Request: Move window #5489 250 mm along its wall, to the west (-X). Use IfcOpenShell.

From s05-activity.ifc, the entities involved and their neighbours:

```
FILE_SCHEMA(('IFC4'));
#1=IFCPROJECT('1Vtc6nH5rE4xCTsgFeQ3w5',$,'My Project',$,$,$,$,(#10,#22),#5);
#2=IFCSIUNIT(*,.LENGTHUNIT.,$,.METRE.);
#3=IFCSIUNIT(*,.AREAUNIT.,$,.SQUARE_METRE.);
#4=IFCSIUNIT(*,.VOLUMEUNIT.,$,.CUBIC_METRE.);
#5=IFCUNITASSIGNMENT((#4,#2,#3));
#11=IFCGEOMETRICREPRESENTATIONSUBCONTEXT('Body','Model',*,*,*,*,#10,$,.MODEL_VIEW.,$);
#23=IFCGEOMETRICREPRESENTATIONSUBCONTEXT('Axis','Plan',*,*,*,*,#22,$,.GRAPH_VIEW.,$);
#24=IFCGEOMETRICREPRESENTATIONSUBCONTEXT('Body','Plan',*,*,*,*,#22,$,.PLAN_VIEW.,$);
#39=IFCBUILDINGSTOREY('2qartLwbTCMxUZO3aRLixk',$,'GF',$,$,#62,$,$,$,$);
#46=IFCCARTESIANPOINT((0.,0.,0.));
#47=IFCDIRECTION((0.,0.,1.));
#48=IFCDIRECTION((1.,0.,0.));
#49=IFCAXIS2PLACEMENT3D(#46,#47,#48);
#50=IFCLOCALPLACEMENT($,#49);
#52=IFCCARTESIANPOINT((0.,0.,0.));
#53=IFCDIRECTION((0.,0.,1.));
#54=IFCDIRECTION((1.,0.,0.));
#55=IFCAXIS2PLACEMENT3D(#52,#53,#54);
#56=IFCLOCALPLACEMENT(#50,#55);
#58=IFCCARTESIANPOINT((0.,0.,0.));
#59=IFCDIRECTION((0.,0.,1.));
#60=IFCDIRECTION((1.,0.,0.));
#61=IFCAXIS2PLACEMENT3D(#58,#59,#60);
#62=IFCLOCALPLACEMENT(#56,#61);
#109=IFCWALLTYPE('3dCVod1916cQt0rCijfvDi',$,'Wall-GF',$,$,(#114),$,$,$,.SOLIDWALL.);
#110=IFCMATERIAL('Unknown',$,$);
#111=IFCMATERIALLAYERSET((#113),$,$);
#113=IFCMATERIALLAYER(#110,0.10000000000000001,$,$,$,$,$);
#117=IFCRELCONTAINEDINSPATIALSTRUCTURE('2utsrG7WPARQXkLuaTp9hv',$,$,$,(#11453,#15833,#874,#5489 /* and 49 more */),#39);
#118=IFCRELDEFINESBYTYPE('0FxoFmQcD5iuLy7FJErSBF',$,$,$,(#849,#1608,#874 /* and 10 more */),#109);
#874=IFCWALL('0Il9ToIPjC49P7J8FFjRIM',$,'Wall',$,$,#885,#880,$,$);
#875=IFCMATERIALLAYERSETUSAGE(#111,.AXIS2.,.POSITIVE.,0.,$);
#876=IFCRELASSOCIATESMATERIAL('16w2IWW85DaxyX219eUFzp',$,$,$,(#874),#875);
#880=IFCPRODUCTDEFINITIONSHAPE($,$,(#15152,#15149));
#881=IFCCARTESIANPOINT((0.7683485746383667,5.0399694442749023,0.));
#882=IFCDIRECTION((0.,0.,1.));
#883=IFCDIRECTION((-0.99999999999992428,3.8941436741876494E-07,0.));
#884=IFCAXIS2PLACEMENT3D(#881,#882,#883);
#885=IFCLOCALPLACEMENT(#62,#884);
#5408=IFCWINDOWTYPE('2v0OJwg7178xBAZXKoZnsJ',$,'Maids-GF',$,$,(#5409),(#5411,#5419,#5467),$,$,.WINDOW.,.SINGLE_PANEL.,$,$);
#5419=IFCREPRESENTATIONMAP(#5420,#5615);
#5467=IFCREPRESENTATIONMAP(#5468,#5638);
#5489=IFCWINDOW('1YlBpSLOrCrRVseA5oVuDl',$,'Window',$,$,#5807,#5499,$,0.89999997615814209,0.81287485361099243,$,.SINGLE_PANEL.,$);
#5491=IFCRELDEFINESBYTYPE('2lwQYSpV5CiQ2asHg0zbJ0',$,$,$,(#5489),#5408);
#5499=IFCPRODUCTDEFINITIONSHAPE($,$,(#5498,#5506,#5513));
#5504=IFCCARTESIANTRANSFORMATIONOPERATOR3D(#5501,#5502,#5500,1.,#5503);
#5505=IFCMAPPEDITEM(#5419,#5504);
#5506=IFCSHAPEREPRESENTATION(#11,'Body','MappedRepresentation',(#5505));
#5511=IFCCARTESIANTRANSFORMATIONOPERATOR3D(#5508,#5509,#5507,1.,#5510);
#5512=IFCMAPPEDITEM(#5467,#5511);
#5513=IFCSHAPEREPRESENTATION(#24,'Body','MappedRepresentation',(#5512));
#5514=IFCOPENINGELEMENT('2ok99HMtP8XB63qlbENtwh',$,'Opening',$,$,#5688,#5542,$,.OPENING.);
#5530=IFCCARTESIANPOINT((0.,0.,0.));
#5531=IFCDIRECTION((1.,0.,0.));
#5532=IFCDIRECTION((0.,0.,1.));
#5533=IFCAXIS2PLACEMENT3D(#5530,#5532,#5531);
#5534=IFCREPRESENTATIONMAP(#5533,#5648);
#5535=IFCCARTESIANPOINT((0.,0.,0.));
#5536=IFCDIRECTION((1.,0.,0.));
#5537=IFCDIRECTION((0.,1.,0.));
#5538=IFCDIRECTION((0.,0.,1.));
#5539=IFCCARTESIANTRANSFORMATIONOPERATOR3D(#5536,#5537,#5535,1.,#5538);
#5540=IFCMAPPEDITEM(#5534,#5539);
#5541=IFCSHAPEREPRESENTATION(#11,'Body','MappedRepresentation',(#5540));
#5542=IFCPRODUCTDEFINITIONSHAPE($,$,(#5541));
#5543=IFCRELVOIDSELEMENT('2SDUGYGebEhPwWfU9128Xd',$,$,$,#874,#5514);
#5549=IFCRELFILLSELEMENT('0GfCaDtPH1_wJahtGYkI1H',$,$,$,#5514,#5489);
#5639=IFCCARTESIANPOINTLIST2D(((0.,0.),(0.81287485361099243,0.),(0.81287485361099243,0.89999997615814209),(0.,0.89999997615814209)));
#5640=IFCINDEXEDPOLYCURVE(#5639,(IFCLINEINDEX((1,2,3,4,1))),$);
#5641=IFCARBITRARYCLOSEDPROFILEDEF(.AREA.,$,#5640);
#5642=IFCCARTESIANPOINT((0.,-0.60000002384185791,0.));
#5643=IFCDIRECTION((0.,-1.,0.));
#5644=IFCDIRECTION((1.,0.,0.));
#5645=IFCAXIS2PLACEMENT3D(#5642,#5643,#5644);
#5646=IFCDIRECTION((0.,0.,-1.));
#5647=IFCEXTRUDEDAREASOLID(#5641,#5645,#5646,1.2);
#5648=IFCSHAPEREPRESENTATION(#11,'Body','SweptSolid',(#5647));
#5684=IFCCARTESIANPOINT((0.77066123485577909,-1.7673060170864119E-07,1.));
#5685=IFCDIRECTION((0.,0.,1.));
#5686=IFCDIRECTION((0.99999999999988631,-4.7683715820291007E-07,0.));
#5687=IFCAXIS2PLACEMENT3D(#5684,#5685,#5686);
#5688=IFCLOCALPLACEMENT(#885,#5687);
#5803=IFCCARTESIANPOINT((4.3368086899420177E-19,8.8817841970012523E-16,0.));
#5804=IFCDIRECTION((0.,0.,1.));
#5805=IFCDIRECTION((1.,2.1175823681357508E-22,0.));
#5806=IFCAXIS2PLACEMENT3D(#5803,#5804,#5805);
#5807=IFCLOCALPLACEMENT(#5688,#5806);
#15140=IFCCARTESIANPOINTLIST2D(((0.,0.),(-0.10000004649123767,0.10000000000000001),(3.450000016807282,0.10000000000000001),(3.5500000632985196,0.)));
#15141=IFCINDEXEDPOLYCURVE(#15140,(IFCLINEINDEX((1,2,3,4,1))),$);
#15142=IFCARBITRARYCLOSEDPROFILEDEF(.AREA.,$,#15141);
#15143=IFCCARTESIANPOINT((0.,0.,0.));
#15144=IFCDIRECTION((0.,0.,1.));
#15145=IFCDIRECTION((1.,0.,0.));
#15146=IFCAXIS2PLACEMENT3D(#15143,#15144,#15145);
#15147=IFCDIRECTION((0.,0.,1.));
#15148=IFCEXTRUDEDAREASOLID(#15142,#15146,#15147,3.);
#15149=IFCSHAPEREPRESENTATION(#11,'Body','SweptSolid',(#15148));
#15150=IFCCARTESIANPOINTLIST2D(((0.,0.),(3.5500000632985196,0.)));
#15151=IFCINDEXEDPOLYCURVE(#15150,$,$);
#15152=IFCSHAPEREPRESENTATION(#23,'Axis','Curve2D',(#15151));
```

```python
import ifcopenshell
import ifcopenshell.api.geometry
import ifcopenshell.util.placement

model = ifcopenshell.open("s05-activity.ifc")

window = model.by_guid("1YlBpSLOrCrRVseA5oVuDl")
opening = window.FillsVoids[0].RelatingOpeningElement
wall = opening.VoidsElements[0].RelatingBuildingElement

wall_matrix = ifcopenshell.util.placement.get_local_placement(wall.ObjectPlacement)
shift = wall_matrix[:3, 0] * 0.25
before = ifcopenshell.util.placement.get_local_placement(window.ObjectPlacement)[:3, 3].copy()

# The window is placed relative to its opening, so it follows when the opening moves.
matrix = ifcopenshell.util.placement.get_local_placement(opening.ObjectPlacement)
matrix[:3, 3] += shift
ifcopenshell.api.geometry.edit_object_placement(
    model, product=opening, matrix=matrix, is_si=False, should_transform_children=True
)

after = ifcopenshell.util.placement.get_local_placement(window.ObjectPlacement)[:3, 3]
print("window moved by", (after - before).round(3) + 0.0)

model.write("s05-activity_v2.ifc")
```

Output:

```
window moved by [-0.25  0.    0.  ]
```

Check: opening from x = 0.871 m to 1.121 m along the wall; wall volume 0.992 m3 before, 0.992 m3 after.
